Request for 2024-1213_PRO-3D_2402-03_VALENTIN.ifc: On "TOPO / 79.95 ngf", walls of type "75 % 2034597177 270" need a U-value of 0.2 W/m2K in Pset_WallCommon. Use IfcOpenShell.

First a look at what the model holds.

```python
import ifcopenshell
import ifcopenshell.util.element

model = ifcopenshell.open("2024-1213_PRO-3D_2402-03_VALENTIN.ifc")
print(model.schema)
storey = next(s for s in model.by_type("IfcBuildingStorey") if s.Name == "TOPO / 79.95 ngf")
walls = [e for e in ifcopenshell.util.element.get_decomposition(storey) if e.is_a("IfcWall")]
seen = {}
for e in walls:
    element_type = ifcopenshell.util.element.get_type(e)
    key = (element_type.Name if element_type != e and element_type else None, ifcopenshell.util.element.get_pset(e, "Pset_WallCommon", "ThermalTransmittance"))
    seen[key] = seen.get(key, 0) + 1
for (name, value), count in sorted(seen.items(), key=str):
    print(count, "x", name, "|", value)
```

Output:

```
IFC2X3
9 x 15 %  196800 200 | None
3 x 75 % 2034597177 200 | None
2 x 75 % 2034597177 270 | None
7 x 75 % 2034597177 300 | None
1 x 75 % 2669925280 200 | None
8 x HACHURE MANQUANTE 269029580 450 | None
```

```python
import ifcopenshell
import ifcopenshell.api.pset
import ifcopenshell.util.element

model = ifcopenshell.open("2024-1213_PRO-3D_2402-03_VALENTIN.ifc")

storey = next(s for s in model.by_type("IfcBuildingStorey") if s.Name == "TOPO / 79.95 ngf")
walls = [e for e in ifcopenshell.util.element.get_decomposition(storey) if e.is_a("IfcWall")]

count = 0
for e in walls:
    element_type = ifcopenshell.util.element.get_type(e)
    if element_type in (None, e) or element_type.Name != "75 % 2034597177 270":
        continue
    # add_pset returns the element's existing set when there is one.
    pset = ifcopenshell.api.pset.add_pset(model, product=e, name="Pset_WallCommon")
    ifcopenshell.api.pset.edit_pset(model, pset=pset, properties={"ThermalTransmittance": 0.2})
    count += 1

print(count, "walls updated")

model.write("2024-1213_PRO-3D_2402-03_VALENTIN_rev.ifc")
```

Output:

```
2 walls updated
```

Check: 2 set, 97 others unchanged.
